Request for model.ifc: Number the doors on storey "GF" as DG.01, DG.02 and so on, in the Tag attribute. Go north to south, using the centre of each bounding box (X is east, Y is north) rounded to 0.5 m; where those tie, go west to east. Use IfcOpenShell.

First a look at what the model holds.

```python
import ifcopenshell
import ifcopenshell.util.element
import ifcopenshell.util.placement

model = ifcopenshell.open("model.ifc")
print(model.schema)
storey = next(s for s in model.by_type("IfcBuildingStorey") if s.Name == "GF")
doors = [e for e in ifcopenshell.util.element.get_decomposition(storey) if e.is_a("IfcDoor")]
for e in sorted(doors, key=lambda e: e.id()):
    origin = ifcopenshell.util.placement.get_local_placement(e.ObjectPlacement)[:3, 3]
    print(e.id(), e.Tag, e.Name, origin.round(2) + 0.0, sep=" | ")
```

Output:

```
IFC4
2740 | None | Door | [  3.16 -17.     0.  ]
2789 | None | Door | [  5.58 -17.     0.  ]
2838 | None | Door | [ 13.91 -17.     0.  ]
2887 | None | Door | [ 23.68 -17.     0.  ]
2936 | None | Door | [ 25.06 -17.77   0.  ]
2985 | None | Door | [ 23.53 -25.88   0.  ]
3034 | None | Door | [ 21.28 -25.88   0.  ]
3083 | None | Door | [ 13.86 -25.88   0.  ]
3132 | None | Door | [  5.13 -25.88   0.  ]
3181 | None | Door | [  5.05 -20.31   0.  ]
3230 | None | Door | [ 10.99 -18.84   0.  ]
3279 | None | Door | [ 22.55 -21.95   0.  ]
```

```python
import ifcopenshell
import ifcopenshell.geom
import ifcopenshell.util.element
import ifcopenshell.util.shape

model = ifcopenshell.open("model.ifc")
settings = ifcopenshell.geom.settings()
settings.set("use-world-coords", True)


def centre(element):
    shape = ifcopenshell.geom.create_shape(settings, element)
    return ifcopenshell.util.shape.get_bbox_centroid(shape.geometry)


storey = next(s for s in model.by_type("IfcBuildingStorey") if s.Name == "GF")
doors = [e for e in ifcopenshell.util.element.get_decomposition(storey) if e.is_a("IfcDoor")]

# Insertion points can sit at a corner or the storey origin, so sort by the geometry (in metres).
centres = {e: centre(e) for e in doors}
doors.sort(key=lambda e: (-round(centres[e][1] / 0.5), centres[e][0]))

for i, e in enumerate(doors, start=1):
    number = f"DG.{i:02d}"
    e.Tag = number
    print(e.id(), number)

model.write("model_v2.ifc")
```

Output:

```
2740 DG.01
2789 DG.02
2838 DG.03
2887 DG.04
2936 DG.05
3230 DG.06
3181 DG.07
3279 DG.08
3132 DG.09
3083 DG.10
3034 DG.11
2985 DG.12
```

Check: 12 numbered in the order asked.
